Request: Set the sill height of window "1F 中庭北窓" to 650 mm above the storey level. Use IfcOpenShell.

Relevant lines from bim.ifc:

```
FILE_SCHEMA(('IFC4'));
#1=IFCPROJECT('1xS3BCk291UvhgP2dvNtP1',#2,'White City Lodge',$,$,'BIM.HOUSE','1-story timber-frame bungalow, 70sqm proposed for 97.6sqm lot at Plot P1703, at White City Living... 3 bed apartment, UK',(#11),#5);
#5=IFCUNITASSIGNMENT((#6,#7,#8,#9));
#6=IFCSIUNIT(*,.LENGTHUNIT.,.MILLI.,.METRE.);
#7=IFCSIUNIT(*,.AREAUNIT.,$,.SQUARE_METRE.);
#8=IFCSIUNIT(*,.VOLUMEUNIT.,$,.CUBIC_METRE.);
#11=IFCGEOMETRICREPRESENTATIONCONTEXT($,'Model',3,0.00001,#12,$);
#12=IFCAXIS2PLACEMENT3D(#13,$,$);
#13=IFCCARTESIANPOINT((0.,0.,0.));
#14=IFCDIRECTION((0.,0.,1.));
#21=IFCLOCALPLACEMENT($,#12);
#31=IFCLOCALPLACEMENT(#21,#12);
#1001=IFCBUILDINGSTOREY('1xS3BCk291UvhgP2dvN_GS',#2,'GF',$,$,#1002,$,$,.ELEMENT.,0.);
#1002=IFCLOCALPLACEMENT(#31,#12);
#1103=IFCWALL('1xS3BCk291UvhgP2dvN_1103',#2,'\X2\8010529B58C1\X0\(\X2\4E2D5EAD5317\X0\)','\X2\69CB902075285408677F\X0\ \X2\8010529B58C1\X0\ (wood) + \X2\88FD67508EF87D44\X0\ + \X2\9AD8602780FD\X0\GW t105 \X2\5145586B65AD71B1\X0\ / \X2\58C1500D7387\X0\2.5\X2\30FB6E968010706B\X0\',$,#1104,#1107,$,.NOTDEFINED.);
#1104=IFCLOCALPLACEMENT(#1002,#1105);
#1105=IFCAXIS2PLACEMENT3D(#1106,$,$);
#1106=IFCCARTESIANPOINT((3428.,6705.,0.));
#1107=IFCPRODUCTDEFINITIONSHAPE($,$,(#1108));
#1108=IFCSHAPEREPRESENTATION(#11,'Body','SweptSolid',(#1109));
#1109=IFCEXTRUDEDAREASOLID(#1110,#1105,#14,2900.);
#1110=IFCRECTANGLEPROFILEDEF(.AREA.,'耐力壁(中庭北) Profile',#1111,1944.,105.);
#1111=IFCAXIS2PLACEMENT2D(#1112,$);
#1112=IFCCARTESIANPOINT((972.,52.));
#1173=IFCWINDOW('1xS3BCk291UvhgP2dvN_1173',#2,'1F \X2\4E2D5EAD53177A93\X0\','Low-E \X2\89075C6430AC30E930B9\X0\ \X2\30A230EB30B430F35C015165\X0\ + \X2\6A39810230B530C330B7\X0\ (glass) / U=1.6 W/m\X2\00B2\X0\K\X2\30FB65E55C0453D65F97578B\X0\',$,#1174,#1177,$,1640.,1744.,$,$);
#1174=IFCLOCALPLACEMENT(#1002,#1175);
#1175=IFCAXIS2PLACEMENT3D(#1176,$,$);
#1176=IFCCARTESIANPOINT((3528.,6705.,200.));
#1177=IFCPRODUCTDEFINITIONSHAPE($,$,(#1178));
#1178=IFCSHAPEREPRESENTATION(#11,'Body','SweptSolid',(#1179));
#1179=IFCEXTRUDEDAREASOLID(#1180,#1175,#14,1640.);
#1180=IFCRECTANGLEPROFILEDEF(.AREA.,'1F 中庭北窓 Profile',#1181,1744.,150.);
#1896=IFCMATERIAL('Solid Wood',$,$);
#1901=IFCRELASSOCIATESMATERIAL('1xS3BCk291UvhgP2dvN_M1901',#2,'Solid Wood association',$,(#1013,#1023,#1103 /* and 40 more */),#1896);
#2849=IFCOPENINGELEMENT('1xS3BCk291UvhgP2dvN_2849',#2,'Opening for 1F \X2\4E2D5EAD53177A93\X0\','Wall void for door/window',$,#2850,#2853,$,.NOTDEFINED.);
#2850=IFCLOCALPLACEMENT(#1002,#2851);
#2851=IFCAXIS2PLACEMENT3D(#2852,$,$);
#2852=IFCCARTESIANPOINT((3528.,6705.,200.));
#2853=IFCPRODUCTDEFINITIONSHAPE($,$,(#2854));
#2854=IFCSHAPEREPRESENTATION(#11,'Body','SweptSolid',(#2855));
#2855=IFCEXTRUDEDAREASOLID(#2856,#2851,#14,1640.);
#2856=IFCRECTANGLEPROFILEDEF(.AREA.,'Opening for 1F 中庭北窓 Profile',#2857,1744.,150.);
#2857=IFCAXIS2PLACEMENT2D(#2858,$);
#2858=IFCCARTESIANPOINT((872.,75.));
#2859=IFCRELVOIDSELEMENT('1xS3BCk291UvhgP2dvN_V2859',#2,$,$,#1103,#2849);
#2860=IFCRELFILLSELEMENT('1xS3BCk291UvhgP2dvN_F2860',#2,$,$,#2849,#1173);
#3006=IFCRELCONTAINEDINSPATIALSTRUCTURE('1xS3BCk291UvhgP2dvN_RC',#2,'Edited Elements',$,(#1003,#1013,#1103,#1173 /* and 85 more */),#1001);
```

```python
import numpy as np
import ifcopenshell
import ifcopenshell.api.geometry
import ifcopenshell.geom
import ifcopenshell.util.element
import ifcopenshell.util.placement
import ifcopenshell.util.shape
import ifcopenshell.util.unit

model = ifcopenshell.open("bim.ifc")
unit_scale = ifcopenshell.util.unit.calculate_unit_scale(model)

window = model.by_id(1173)
opening = window.FillsVoids[0].RelatingOpeningElement
storey = ifcopenshell.util.element.get_container(window, ifc_class="IfcBuildingStorey")
level = ifcopenshell.util.placement.get_local_placement(storey.ObjectPlacement)[2, 3]

# The opening's origin need not be at the sill, so measure its lowest point.
shape = ifcopenshell.geom.create_shape(ifcopenshell.geom.settings(), opening)
bottom = ifcopenshell.util.shape.get_shape_bottom_elevation(shape, shape.geometry) / unit_scale
dz = level + 0.65 / unit_scale - bottom

shift = np.array([0.0, 0.0, dz])
# The window is not placed relative to its opening, so move both.
for product in (opening, window):
    matrix = ifcopenshell.util.placement.get_local_placement(product.ObjectPlacement)
    matrix[:3, 3] += shift
    ifcopenshell.api.geometry.edit_object_placement(model, product=product, matrix=matrix, is_si=False)

print(f"moved by {dz * unit_scale:+.3f} m")

model.write("bim_updated.ifc")
```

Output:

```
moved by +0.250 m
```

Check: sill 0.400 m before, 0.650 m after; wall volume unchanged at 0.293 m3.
